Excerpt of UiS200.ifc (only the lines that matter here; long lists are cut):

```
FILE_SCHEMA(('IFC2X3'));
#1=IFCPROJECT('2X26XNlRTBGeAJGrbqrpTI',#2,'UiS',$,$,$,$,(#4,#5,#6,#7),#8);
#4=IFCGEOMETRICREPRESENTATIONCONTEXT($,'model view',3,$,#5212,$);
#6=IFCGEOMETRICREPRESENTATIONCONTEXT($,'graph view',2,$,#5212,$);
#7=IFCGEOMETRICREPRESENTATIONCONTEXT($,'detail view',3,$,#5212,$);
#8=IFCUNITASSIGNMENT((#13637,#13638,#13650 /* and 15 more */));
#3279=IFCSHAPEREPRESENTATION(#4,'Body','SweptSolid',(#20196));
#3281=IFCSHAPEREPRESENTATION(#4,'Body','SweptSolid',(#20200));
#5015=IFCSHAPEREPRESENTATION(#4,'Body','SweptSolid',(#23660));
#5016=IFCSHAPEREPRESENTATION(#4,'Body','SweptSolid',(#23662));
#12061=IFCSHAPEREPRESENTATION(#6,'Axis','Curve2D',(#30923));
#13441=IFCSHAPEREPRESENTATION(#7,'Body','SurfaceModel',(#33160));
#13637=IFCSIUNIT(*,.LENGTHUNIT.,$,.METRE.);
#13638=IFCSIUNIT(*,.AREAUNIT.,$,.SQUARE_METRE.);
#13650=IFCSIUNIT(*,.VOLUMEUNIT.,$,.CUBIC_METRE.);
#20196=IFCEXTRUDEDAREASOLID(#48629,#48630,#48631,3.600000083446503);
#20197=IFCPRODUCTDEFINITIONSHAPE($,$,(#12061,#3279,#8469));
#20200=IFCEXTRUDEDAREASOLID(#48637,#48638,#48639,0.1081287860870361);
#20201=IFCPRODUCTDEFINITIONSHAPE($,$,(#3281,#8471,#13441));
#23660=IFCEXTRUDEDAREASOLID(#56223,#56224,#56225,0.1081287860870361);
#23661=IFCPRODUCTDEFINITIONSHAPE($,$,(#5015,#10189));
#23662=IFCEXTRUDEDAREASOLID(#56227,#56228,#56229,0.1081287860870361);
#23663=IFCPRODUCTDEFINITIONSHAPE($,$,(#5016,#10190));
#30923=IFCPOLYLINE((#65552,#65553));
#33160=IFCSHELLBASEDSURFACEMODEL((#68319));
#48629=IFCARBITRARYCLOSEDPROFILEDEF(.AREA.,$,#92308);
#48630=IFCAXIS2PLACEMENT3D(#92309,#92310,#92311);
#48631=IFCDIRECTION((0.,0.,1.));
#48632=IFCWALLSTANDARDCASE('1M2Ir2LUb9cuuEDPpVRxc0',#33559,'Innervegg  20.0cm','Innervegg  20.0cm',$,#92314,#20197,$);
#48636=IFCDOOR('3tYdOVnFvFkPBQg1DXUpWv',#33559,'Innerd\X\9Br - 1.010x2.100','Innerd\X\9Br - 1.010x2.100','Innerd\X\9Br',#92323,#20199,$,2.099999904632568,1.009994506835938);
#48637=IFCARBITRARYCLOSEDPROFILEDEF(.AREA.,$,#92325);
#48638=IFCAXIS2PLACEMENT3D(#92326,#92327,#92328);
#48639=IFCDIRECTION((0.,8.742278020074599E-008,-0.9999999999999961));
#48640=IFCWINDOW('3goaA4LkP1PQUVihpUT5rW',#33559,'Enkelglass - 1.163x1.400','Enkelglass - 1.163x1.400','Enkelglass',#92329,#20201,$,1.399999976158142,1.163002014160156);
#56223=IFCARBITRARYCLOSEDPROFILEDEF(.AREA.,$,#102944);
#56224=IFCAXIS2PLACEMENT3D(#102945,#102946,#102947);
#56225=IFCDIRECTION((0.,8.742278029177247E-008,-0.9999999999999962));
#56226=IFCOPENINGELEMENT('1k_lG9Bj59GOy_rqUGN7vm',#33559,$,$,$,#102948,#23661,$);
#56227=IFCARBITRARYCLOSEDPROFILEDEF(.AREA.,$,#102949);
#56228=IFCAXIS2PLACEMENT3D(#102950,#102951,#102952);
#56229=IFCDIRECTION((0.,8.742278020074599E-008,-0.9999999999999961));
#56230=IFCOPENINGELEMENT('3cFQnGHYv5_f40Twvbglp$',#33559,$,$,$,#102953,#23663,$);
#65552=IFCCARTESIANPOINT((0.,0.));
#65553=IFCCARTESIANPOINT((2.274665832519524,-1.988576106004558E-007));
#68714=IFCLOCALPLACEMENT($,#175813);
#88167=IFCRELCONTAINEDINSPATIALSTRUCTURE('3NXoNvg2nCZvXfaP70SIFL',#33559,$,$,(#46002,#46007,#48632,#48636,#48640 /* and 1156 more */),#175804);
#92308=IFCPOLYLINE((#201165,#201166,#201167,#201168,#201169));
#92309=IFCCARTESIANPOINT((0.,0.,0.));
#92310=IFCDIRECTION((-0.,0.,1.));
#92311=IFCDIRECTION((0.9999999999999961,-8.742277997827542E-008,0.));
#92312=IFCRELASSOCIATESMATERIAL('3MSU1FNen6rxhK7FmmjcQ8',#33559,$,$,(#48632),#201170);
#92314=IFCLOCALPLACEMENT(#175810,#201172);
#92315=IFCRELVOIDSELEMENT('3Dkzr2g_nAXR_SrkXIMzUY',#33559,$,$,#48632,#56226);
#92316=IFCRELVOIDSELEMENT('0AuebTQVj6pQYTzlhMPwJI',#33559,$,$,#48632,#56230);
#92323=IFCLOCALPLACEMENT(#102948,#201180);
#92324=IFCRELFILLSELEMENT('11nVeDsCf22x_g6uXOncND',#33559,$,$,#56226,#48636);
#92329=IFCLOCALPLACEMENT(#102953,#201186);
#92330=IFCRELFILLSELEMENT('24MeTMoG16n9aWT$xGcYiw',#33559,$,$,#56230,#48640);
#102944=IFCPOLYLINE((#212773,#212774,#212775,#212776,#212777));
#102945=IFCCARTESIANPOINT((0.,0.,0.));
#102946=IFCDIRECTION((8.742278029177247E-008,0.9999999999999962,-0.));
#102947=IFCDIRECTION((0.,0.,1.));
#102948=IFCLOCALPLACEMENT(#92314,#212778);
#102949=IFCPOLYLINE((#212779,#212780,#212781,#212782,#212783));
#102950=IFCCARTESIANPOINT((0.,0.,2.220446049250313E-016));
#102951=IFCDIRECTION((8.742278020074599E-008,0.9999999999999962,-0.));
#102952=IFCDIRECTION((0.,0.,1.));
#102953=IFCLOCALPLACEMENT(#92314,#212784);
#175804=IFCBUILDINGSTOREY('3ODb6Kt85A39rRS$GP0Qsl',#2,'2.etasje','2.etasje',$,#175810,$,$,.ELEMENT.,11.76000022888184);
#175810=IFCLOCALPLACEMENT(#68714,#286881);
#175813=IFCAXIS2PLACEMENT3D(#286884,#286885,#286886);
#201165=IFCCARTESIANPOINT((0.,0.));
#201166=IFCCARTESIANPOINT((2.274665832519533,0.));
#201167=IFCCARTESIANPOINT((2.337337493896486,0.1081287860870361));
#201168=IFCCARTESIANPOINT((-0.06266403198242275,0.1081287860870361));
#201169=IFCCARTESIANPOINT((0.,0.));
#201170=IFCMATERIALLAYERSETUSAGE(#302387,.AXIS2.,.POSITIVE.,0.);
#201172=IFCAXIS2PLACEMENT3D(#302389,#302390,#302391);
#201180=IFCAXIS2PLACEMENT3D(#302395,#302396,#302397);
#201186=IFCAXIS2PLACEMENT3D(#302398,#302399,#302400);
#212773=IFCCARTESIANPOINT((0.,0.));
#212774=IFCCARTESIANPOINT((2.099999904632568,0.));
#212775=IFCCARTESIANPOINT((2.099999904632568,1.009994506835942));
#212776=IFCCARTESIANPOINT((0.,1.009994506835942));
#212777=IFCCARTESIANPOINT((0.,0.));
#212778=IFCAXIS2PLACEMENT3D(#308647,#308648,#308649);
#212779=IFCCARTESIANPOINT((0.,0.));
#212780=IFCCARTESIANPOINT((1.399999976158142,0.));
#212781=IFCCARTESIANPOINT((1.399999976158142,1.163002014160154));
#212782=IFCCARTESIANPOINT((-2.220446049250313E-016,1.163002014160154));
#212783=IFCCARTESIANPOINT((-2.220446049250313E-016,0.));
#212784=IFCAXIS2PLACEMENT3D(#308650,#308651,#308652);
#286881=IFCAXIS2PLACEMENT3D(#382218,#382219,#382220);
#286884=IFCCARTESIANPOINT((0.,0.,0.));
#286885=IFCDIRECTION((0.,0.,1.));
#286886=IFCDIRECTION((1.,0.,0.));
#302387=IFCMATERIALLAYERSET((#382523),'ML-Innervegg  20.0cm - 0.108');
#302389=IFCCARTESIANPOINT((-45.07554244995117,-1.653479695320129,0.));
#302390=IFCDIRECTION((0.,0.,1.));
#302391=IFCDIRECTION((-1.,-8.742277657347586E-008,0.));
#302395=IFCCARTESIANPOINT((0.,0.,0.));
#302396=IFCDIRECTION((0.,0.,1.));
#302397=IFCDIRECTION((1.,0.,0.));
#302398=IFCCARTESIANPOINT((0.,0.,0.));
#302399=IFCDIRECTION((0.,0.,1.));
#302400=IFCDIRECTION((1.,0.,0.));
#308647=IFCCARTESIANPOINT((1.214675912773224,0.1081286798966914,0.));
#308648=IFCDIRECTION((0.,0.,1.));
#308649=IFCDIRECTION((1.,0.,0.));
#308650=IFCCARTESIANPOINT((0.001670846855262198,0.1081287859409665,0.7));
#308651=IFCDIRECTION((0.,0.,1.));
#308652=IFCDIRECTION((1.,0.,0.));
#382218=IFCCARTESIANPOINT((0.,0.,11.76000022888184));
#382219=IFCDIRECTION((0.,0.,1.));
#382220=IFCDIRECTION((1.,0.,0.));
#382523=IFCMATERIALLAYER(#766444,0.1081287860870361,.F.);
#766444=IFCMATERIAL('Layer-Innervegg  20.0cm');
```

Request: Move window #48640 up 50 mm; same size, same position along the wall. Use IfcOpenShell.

```python
import numpy as np
import ifcopenshell
import ifcopenshell.api.geometry
import ifcopenshell.util.placement
import ifcopenshell.util.unit

model = ifcopenshell.open("UiS200.ifc")
unit_scale = ifcopenshell.util.unit.calculate_unit_scale(model)

window = model.by_guid("3goaA4LkP1PQUVihpUT5rW")
opening = window.FillsVoids[0].RelatingOpeningElement
dz = 0.05 / unit_scale

shift = np.array([0.0, 0.0, dz])
# The window is placed relative to its opening, so it follows when the opening moves.
matrix = ifcopenshell.util.placement.get_local_placement(opening.ObjectPlacement)
matrix[:3, 3] += shift
ifcopenshell.api.geometry.edit_object_placement(
    model, product=opening, matrix=matrix, is_si=False, should_transform_children=True
)

print(f"moved by {dz * unit_scale:+.3f} m")

model.write("UiS200_v2.ifc")
```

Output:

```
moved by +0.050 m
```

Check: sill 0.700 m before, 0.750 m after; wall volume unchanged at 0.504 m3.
